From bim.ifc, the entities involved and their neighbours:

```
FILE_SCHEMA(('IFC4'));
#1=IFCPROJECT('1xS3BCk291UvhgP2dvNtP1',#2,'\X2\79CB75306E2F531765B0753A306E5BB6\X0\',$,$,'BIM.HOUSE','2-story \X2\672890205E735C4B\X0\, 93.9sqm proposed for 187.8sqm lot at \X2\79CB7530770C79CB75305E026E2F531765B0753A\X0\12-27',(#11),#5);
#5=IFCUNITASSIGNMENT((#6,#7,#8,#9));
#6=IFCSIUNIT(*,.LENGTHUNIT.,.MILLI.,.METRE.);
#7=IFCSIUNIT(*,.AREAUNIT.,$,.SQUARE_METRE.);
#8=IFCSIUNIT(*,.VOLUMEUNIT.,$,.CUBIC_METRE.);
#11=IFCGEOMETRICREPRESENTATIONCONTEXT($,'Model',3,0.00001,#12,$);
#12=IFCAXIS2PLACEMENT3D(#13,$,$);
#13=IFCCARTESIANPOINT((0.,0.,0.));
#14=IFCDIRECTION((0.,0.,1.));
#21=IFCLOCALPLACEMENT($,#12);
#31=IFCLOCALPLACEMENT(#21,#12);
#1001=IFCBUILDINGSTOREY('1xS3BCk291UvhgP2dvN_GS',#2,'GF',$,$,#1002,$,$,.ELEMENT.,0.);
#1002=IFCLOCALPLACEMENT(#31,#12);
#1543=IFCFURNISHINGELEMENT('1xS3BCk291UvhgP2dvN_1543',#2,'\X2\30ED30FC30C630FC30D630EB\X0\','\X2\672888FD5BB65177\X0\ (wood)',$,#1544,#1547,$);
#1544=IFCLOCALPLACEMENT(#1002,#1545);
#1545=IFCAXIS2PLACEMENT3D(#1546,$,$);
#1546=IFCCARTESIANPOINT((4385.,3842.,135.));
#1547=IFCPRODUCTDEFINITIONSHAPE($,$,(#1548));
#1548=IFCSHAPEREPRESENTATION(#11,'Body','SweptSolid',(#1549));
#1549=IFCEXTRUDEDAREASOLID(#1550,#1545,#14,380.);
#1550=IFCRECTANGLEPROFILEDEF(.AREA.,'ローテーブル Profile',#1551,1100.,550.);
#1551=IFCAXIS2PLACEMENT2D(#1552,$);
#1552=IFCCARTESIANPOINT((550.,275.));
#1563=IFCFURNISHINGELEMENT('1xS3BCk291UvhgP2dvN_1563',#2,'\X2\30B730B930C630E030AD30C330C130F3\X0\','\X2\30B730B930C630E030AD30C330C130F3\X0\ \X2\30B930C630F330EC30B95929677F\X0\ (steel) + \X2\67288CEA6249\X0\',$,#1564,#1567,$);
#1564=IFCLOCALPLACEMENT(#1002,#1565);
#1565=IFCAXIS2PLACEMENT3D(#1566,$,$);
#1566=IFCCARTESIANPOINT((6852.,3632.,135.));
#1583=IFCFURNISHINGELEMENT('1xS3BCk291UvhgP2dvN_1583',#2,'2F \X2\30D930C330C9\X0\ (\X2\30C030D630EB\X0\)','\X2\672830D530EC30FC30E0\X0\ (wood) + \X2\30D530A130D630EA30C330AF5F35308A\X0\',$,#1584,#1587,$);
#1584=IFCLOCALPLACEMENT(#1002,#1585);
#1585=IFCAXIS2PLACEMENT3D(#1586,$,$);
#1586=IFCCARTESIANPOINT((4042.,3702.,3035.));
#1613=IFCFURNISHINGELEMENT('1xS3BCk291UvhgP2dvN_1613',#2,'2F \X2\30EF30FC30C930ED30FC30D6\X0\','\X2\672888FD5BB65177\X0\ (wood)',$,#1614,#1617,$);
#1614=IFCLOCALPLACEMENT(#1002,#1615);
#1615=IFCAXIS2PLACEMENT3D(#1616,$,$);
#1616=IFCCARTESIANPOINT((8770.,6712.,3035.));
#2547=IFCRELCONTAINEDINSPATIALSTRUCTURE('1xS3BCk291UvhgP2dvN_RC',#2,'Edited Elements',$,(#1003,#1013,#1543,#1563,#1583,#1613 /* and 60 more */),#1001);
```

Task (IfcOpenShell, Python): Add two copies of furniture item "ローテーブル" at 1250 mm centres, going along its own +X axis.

```python
import ifcopenshell
import ifcopenshell.api.geometry
import ifcopenshell.api.root
import ifcopenshell.util.element
import ifcopenshell.util.placement
import ifcopenshell.util.unit

model = ifcopenshell.open("bim.ifc")
unit_scale = ifcopenshell.util.unit.calculate_unit_scale(model)


def reuse_history(source, copy):
    """copy_class also copies each property set's owner history, people and application; keep the originals."""
    for rel in copy.IsDefinedBy:
        if rel.is_a("IfcRelDefinesByProperties") and (history := rel.RelatingPropertyDefinition.OwnerHistory):
            rel.RelatingPropertyDefinition.OwnerHistory = source.OwnerHistory
            ifcopenshell.util.element.remove_deep2(model, history)


source = model.by_guid("1xS3BCk291UvhgP2dvN_1543")
base = ifcopenshell.util.placement.get_local_placement(source.ObjectPlacement)
step = base[:3, 0] * 1.25 / unit_scale

for i in range(1, 3):
    copy = ifcopenshell.api.root.copy_class(model, product=source)
    copy.Representation = ifcopenshell.util.element.copy_deep(
        model, source.Representation, exclude=["IfcGeometricRepresentationContext", "IfcRepresentationMap"]
    )
    reuse_history(source, copy)
    matrix = base.copy()
    matrix[:3, 3] += i * step
    print("added at", matrix[:3, 3].round(3) + 0.0)
    ifcopenshell.api.geometry.edit_object_placement(model, product=copy, matrix=matrix, is_si=False)

model.write("bim_rev.ifc")
```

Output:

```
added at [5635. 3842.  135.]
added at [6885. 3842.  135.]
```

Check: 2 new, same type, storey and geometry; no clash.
